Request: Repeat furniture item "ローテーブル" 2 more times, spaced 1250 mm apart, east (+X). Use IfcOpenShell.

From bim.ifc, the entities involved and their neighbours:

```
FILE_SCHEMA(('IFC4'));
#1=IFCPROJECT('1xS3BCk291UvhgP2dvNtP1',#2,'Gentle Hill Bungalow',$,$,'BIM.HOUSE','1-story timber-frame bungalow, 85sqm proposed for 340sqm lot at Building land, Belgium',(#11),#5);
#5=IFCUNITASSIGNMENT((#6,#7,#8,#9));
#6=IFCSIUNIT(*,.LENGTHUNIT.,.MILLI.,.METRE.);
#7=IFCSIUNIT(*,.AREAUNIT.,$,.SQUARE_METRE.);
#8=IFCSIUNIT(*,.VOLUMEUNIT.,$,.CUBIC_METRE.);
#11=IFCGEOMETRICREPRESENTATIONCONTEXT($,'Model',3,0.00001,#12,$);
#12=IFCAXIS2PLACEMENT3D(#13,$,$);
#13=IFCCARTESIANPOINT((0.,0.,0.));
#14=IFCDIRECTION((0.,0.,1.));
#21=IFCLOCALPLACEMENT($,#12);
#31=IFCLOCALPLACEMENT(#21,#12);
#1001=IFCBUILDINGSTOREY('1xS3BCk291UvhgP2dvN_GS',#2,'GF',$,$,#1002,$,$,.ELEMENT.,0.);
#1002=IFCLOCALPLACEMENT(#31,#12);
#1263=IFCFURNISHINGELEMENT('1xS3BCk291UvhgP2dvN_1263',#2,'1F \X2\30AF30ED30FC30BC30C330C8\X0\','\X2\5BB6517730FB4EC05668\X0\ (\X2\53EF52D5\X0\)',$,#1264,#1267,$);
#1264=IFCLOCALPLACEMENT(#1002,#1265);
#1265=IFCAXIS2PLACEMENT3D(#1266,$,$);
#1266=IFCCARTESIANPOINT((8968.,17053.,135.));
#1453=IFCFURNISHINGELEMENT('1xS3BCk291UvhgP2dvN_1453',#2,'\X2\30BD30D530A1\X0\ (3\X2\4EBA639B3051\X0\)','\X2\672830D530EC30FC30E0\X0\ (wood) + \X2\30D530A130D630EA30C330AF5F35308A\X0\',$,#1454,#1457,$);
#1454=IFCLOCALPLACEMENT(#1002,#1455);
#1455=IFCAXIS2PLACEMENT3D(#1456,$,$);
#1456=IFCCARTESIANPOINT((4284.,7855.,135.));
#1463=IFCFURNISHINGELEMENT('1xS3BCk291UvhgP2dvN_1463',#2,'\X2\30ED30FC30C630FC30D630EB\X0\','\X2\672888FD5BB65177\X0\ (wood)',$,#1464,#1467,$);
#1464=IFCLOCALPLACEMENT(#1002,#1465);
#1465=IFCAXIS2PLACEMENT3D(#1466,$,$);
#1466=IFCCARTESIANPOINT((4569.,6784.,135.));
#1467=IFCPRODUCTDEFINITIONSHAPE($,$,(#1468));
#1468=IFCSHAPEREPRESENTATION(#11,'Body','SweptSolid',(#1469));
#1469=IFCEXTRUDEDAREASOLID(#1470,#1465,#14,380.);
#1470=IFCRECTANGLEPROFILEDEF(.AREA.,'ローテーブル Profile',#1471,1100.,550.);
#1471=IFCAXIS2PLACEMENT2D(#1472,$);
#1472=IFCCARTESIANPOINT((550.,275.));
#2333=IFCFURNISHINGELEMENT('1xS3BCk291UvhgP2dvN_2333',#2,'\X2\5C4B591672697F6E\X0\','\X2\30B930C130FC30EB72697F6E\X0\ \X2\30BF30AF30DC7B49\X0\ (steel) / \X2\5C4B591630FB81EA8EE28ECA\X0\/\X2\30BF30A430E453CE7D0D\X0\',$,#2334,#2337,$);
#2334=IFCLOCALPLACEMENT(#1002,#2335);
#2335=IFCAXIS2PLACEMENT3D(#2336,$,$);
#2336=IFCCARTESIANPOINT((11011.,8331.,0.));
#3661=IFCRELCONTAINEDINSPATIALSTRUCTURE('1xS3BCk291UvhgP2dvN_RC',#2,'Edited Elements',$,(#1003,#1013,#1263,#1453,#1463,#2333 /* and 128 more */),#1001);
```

```python
import numpy as np
import ifcopenshell
import ifcopenshell.api.geometry
import ifcopenshell.api.root
import ifcopenshell.util.element
import ifcopenshell.util.placement

model = ifcopenshell.open("bim.ifc")


def reuse_history(source, copy):
    """copy_class also copies each property set's owner history, people and application; keep the originals."""
    for rel in copy.IsDefinedBy:
        if rel.is_a("IfcRelDefinesByProperties") and (history := rel.RelatingPropertyDefinition.OwnerHistory):
            rel.RelatingPropertyDefinition.OwnerHistory = source.OwnerHistory
            ifcopenshell.util.element.remove_deep2(model, history)


source = model.by_guid("1xS3BCk291UvhgP2dvN_1463")
base = ifcopenshell.util.placement.get_local_placement(source.ObjectPlacement)
step = np.array([1.0, 0.0, 0.0]) * 1250.0

for i in range(1, 3):
    copy = ifcopenshell.api.root.copy_class(model, product=source)
    copy.Representation = ifcopenshell.util.element.copy_deep(
        model, source.Representation, exclude=["IfcGeometricRepresentationContext", "IfcRepresentationMap"]
    )
    reuse_history(source, copy)
    matrix = base.copy()
    matrix[:3, 3] += i * step
    print("added at", matrix[:3, 3].round(3) + 0.0)
    ifcopenshell.api.geometry.edit_object_placement(model, product=copy, matrix=matrix, is_si=False)

model.write("bim_rev.ifc")
```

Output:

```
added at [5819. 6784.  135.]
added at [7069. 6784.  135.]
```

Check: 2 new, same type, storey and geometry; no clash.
